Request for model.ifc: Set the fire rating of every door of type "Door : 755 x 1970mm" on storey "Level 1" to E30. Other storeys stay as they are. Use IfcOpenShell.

First a look at what the model holds.

```python
import ifcopenshell
import ifcopenshell.util.element

model = ifcopenshell.open("model.ifc")
print(model.schema)
storey = next(s for s in model.by_type("IfcBuildingStorey") if s.Name == "Level 1")
doors = [e for e in ifcopenshell.util.element.get_decomposition(storey) if e.is_a("IfcDoor")]
seen = {}
for e in doors:
    element_type = ifcopenshell.util.element.get_type(e)
    key = (element_type.Name if element_type != e and element_type else None, ifcopenshell.util.element.get_pset(e, "Pset_DoorCommon", "FireRating"))
    seen[key] = seen.get(key, 0) + 1
for (name, value), count in sorted(seen.items(), key=str):
    print(count, "x", name, "|", value)
```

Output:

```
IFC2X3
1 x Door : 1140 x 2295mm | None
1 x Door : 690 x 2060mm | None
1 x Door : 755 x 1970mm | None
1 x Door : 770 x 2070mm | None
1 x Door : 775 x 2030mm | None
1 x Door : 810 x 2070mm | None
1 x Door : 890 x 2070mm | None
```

```python
import ifcopenshell
import ifcopenshell.api.pset
import ifcopenshell.util.element

model = ifcopenshell.open("model.ifc")

storey = next(s for s in model.by_type("IfcBuildingStorey") if s.Name == "Level 1")
doors = [e for e in ifcopenshell.util.element.get_decomposition(storey) if e.is_a("IfcDoor")]

count = 0
for e in doors:
    element_type = ifcopenshell.util.element.get_type(e)
    if element_type in (None, e) or element_type.Name != "Door : 755 x 1970mm":
        continue
    # add_pset returns the element's existing set when there is one.
    pset = ifcopenshell.api.pset.add_pset(model, product=e, name="Pset_DoorCommon")
    ifcopenshell.api.pset.edit_pset(model, pset=pset, properties={"FireRating": "E30"})
    count += 1

print(count, "doors updated")

model.write("model_v2.ifc")
```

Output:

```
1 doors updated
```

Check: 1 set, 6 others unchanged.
